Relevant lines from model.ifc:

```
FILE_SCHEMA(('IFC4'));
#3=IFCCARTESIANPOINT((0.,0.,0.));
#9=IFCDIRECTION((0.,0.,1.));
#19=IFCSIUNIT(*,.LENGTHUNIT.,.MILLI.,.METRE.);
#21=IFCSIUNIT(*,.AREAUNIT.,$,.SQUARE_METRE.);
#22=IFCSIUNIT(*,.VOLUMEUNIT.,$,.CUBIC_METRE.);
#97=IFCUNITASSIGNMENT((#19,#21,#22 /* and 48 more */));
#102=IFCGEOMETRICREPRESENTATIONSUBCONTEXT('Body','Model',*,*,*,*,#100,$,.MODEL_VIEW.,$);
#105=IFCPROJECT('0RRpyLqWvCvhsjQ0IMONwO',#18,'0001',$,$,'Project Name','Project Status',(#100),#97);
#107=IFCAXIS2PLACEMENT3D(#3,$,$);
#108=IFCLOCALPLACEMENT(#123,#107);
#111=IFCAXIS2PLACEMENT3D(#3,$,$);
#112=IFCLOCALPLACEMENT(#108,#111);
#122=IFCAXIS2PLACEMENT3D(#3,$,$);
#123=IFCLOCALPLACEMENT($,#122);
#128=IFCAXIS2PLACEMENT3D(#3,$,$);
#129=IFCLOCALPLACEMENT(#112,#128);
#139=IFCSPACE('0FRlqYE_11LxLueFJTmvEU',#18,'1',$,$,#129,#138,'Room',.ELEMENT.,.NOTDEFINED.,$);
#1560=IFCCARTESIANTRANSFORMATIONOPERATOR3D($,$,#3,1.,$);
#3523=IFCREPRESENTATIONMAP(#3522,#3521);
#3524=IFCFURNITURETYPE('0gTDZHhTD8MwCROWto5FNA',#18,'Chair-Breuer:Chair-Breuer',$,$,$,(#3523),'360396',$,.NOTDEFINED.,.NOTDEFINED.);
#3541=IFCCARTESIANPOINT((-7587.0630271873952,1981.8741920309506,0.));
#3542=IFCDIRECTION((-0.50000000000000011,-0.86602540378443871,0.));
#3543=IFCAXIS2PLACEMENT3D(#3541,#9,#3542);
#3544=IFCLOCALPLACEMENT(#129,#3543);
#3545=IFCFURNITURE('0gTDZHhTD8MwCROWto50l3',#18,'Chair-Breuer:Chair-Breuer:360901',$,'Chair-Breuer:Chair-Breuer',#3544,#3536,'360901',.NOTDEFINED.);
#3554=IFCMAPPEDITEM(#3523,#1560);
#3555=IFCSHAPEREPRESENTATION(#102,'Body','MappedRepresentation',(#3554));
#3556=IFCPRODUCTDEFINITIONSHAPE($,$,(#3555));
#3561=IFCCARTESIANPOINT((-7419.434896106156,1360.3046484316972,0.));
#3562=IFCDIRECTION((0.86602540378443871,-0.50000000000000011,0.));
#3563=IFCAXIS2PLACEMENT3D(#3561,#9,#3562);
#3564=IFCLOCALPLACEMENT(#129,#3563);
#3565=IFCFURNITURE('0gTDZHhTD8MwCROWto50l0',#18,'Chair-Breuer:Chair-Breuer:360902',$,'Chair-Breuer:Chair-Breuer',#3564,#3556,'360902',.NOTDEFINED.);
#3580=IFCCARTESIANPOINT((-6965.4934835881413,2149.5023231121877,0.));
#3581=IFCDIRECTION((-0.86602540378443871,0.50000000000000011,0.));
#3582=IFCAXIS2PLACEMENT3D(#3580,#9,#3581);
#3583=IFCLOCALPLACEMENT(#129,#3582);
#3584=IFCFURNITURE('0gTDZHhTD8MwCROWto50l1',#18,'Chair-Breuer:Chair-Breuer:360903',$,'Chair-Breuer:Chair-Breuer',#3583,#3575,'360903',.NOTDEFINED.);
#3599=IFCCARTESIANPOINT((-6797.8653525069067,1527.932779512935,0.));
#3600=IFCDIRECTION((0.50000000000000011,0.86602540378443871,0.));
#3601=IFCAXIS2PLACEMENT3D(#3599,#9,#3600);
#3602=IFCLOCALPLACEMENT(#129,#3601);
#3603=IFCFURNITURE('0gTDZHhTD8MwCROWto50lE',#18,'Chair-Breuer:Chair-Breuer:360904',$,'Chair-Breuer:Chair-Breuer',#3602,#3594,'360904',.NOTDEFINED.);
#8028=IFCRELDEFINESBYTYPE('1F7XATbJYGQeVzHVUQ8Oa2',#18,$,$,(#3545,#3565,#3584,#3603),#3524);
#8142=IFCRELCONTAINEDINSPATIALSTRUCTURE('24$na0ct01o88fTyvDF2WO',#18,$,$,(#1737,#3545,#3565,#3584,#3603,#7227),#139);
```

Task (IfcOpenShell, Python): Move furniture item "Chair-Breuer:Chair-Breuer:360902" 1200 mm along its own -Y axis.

```python
import ifcopenshell
import ifcopenshell.api.geometry
import ifcopenshell.util.placement

model = ifcopenshell.open("model.ifc")

item = model.by_guid("0gTDZHhTD8MwCROWto50l0")
matrix = ifcopenshell.util.placement.get_local_placement(item.ObjectPlacement)
matrix[:3, 3] -= matrix[:3, 1] * 1200.0
ifcopenshell.api.geometry.edit_object_placement(model, product=item, matrix=matrix, is_si=False)

print(ifcopenshell.util.placement.get_local_placement(item.ObjectPlacement).round(3) + 0.0)

model.write("model-out.ifc")
```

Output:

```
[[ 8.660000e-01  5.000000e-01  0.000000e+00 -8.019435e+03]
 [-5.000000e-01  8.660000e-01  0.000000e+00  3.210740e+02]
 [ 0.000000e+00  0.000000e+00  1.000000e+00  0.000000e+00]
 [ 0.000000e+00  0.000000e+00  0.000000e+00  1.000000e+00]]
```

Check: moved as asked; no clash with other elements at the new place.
